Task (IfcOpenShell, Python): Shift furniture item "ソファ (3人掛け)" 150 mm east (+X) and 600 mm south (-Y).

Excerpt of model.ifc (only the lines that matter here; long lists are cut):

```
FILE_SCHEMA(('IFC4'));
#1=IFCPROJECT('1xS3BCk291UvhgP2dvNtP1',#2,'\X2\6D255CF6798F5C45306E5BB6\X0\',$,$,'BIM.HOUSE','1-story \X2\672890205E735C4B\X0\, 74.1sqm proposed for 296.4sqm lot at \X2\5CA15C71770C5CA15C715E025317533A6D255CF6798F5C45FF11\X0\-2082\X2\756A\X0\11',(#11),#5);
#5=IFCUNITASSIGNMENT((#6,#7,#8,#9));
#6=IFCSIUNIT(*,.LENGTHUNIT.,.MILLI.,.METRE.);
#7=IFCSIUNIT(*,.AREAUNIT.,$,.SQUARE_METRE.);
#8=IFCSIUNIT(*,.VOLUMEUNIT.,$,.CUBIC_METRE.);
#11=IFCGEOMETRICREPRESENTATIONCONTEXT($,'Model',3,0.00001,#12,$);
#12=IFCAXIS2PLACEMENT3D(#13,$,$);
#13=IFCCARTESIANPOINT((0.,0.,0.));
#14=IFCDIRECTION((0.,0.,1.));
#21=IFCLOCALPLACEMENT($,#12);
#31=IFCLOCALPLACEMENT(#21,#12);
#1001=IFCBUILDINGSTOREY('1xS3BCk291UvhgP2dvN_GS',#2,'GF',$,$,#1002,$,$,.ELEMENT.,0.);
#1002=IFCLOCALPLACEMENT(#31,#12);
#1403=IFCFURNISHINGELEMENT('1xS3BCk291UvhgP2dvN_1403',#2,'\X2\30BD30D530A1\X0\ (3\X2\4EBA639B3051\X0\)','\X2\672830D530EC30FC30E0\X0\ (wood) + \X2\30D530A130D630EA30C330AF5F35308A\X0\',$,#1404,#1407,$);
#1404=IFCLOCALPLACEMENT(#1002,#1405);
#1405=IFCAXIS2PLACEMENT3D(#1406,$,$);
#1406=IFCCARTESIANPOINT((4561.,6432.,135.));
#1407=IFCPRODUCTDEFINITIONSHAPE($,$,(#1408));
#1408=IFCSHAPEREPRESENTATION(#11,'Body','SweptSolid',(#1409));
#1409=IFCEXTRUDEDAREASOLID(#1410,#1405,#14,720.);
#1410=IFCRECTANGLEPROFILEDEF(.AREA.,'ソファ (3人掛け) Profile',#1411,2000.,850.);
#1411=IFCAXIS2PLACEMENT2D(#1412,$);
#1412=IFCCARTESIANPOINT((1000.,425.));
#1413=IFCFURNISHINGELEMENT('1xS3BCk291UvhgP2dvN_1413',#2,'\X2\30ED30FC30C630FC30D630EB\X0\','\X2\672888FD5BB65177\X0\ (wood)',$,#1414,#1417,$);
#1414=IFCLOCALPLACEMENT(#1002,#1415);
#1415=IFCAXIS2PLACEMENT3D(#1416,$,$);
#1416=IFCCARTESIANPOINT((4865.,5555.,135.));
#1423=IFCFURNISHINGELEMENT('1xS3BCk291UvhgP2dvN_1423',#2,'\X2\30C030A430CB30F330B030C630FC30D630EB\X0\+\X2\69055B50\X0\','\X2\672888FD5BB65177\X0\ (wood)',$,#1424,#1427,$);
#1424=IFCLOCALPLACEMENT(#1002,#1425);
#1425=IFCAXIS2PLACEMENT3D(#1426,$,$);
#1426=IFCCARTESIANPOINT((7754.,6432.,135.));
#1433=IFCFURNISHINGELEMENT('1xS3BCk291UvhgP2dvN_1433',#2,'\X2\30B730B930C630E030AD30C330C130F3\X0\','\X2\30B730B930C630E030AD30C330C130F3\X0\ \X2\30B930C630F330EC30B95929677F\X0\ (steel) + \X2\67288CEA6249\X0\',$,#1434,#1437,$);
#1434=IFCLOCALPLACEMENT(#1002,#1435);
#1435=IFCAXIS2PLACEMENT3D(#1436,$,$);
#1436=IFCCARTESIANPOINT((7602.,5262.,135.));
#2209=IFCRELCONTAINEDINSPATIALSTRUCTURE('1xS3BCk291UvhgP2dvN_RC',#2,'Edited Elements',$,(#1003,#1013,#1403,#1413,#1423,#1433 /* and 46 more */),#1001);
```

```python
import ifcopenshell
import ifcopenshell.api.geometry
import ifcopenshell.util.placement
import ifcopenshell.util.unit

model = ifcopenshell.open("model.ifc")
unit_scale = ifcopenshell.util.unit.calculate_unit_scale(model)

item = model.by_guid("1xS3BCk291UvhgP2dvN_1403")
matrix = ifcopenshell.util.placement.get_local_placement(item.ObjectPlacement)
matrix[0, 3] += 0.15 / unit_scale
matrix[1, 3] -= 0.6 / unit_scale
ifcopenshell.api.geometry.edit_object_placement(model, product=item, matrix=matrix, is_si=False)

print(ifcopenshell.util.placement.get_local_placement(item.ObjectPlacement).round(3) + 0.0)

model.write("model_updated.ifc")
```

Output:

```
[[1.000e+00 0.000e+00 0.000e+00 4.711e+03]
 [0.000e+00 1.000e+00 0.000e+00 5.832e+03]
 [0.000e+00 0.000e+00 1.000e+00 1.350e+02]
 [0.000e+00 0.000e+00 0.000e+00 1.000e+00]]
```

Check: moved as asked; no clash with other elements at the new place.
